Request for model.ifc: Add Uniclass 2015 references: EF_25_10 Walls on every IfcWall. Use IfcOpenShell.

First a look at what the model holds.

```python
import ifcopenshell

model = ifcopenshell.open("model.ifc")
print(model.schema)
print("classifications:", [c.Name for c in model.by_type("IfcClassification")])
for ifc_class in ("IfcDoor", "IfcRoof", "IfcStair", "IfcWall", "IfcWindow"):
    print(ifc_class, len(model.by_type(ifc_class)))
```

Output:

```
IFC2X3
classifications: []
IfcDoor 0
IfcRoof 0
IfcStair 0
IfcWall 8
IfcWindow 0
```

```python
import ifcopenshell
import ifcopenshell.api.classification

model = ifcopenshell.open("model.ifc")

# IFC2X3 requires Source and Edition and has no link from the project to the system.
system = model.create_entity("IfcClassification", Source="NBS", Edition="2015", Name="Uniclass 2015")

codes = {
    "IfcWall": ("EF_25_10", "Walls"),
}
for ifc_class, (code, name) in codes.items():
    products = model.by_type(ifc_class)
    ifcopenshell.api.classification.add_reference(
        model, products=products, classification=system, identification=code, name=name
    )
    print(code, len(products))

model.write("model_updated.ifc")
```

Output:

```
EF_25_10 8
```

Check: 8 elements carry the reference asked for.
